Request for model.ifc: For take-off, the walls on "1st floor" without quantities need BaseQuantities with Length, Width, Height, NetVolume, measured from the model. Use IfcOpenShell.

First a look at what the model holds.

```python
import ifcopenshell
import ifcopenshell.util.element
import ifcopenshell.util.unit

model = ifcopenshell.open("model.ifc")
print(model.schema)
for unit_type in ("LENGTHUNIT", "AREAUNIT", "VOLUMEUNIT"):
    print(unit_type, ifcopenshell.util.unit.calculate_unit_scale(model, unit_type))
storey = next(s for s in model.by_type("IfcBuildingStorey") if s.Name == "1st floor")
walls = [e for e in ifcopenshell.util.element.get_decomposition(storey) if e.is_a("IfcWall")]
for e in sorted(walls, key=lambda e: e.id()):
    print(e.id(), e.is_a(), e.Name, list(ifcopenshell.util.element.get_psets(e, qtos_only=True)), sep=" | ")
```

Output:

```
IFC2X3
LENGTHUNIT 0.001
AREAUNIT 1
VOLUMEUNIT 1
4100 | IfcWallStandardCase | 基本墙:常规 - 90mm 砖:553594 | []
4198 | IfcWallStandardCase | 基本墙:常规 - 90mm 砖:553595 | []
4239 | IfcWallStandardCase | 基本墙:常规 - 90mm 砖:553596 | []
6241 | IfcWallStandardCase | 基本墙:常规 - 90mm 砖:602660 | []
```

```python
import ifcopenshell
import ifcopenshell.api.pset
import ifcopenshell.geom
import ifcopenshell.util.element
import ifcopenshell.util.shape
import ifcopenshell.util.unit

model = ifcopenshell.open("model.ifc")
unit_scale = ifcopenshell.util.unit.calculate_unit_scale(model)
volume_scale = ifcopenshell.util.unit.calculate_unit_scale(model, "VOLUMEUNIT")
settings = ifcopenshell.geom.settings()

storey = next(s for s in model.by_type("IfcBuildingStorey") if s.Name == "1st floor")
walls = [e for e in ifcopenshell.util.element.get_decomposition(storey) if e.is_a("IfcWall")]

for e in sorted(walls, key=lambda e: e.id()):
    if ifcopenshell.util.element.get_psets(e, qtos_only=True, should_inherit=False):
        continue
    # Geometry comes back in metres, in the element's own axes.
    shape = ifcopenshell.geom.create_shape(settings, e)
    values = {
        "Length": ifcopenshell.util.shape.get_x(shape.geometry) / unit_scale,
        "Width": ifcopenshell.util.shape.get_y(shape.geometry) / unit_scale,
        "Height": ifcopenshell.util.shape.get_z(shape.geometry) / unit_scale,
        "NetVolume": ifcopenshell.util.shape.get_volume(shape.geometry) / volume_scale,
    }
    qto = ifcopenshell.api.pset.add_qto(model, product=e, name="BaseQuantities")
    ifcopenshell.api.pset.edit_qto(model, qto=qto, properties=values)
    print(e.id(), {k: round(v, 3) for k, v in values.items()})

model.write("model_v2.ifc")
```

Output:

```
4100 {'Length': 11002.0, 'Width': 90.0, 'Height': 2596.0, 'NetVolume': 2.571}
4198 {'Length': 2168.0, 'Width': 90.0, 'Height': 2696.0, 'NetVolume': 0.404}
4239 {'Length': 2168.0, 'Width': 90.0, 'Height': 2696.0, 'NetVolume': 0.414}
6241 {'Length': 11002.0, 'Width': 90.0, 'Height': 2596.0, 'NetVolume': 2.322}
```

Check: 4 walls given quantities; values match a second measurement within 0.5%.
